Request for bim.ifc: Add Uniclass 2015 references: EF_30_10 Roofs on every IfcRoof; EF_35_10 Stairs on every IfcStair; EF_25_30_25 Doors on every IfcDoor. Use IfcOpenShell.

First a look at what the model holds.

```python
import ifcopenshell

model = ifcopenshell.open("bim.ifc")
print(model.schema)
print("classifications:", [c.Name for c in model.by_type("IfcClassification")])
for ifc_class in ("IfcDoor", "IfcRoof", "IfcStair", "IfcWall", "IfcWindow"):
    print(ifc_class, len(model.by_type(ifc_class)))
```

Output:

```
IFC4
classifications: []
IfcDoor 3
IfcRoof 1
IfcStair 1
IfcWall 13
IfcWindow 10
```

```python
import ifcopenshell
import ifcopenshell.api.classification

model = ifcopenshell.open("bim.ifc")

system = ifcopenshell.api.classification.add_classification(model, classification="Uniclass 2015")

codes = {
    "IfcRoof": ("EF_30_10", "Roofs"),
    "IfcStair": ("EF_35_10", "Stairs"),
    "IfcDoor": ("EF_25_30_25", "Doors"),
}
for ifc_class, (code, name) in codes.items():
    products = model.by_type(ifc_class)
    ifcopenshell.api.classification.add_reference(
        model, products=products, classification=system, identification=code, name=name
    )
    print(code, len(products))

model.write("bim_rev.ifc")
```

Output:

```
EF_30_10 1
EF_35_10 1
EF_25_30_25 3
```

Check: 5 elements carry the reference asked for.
